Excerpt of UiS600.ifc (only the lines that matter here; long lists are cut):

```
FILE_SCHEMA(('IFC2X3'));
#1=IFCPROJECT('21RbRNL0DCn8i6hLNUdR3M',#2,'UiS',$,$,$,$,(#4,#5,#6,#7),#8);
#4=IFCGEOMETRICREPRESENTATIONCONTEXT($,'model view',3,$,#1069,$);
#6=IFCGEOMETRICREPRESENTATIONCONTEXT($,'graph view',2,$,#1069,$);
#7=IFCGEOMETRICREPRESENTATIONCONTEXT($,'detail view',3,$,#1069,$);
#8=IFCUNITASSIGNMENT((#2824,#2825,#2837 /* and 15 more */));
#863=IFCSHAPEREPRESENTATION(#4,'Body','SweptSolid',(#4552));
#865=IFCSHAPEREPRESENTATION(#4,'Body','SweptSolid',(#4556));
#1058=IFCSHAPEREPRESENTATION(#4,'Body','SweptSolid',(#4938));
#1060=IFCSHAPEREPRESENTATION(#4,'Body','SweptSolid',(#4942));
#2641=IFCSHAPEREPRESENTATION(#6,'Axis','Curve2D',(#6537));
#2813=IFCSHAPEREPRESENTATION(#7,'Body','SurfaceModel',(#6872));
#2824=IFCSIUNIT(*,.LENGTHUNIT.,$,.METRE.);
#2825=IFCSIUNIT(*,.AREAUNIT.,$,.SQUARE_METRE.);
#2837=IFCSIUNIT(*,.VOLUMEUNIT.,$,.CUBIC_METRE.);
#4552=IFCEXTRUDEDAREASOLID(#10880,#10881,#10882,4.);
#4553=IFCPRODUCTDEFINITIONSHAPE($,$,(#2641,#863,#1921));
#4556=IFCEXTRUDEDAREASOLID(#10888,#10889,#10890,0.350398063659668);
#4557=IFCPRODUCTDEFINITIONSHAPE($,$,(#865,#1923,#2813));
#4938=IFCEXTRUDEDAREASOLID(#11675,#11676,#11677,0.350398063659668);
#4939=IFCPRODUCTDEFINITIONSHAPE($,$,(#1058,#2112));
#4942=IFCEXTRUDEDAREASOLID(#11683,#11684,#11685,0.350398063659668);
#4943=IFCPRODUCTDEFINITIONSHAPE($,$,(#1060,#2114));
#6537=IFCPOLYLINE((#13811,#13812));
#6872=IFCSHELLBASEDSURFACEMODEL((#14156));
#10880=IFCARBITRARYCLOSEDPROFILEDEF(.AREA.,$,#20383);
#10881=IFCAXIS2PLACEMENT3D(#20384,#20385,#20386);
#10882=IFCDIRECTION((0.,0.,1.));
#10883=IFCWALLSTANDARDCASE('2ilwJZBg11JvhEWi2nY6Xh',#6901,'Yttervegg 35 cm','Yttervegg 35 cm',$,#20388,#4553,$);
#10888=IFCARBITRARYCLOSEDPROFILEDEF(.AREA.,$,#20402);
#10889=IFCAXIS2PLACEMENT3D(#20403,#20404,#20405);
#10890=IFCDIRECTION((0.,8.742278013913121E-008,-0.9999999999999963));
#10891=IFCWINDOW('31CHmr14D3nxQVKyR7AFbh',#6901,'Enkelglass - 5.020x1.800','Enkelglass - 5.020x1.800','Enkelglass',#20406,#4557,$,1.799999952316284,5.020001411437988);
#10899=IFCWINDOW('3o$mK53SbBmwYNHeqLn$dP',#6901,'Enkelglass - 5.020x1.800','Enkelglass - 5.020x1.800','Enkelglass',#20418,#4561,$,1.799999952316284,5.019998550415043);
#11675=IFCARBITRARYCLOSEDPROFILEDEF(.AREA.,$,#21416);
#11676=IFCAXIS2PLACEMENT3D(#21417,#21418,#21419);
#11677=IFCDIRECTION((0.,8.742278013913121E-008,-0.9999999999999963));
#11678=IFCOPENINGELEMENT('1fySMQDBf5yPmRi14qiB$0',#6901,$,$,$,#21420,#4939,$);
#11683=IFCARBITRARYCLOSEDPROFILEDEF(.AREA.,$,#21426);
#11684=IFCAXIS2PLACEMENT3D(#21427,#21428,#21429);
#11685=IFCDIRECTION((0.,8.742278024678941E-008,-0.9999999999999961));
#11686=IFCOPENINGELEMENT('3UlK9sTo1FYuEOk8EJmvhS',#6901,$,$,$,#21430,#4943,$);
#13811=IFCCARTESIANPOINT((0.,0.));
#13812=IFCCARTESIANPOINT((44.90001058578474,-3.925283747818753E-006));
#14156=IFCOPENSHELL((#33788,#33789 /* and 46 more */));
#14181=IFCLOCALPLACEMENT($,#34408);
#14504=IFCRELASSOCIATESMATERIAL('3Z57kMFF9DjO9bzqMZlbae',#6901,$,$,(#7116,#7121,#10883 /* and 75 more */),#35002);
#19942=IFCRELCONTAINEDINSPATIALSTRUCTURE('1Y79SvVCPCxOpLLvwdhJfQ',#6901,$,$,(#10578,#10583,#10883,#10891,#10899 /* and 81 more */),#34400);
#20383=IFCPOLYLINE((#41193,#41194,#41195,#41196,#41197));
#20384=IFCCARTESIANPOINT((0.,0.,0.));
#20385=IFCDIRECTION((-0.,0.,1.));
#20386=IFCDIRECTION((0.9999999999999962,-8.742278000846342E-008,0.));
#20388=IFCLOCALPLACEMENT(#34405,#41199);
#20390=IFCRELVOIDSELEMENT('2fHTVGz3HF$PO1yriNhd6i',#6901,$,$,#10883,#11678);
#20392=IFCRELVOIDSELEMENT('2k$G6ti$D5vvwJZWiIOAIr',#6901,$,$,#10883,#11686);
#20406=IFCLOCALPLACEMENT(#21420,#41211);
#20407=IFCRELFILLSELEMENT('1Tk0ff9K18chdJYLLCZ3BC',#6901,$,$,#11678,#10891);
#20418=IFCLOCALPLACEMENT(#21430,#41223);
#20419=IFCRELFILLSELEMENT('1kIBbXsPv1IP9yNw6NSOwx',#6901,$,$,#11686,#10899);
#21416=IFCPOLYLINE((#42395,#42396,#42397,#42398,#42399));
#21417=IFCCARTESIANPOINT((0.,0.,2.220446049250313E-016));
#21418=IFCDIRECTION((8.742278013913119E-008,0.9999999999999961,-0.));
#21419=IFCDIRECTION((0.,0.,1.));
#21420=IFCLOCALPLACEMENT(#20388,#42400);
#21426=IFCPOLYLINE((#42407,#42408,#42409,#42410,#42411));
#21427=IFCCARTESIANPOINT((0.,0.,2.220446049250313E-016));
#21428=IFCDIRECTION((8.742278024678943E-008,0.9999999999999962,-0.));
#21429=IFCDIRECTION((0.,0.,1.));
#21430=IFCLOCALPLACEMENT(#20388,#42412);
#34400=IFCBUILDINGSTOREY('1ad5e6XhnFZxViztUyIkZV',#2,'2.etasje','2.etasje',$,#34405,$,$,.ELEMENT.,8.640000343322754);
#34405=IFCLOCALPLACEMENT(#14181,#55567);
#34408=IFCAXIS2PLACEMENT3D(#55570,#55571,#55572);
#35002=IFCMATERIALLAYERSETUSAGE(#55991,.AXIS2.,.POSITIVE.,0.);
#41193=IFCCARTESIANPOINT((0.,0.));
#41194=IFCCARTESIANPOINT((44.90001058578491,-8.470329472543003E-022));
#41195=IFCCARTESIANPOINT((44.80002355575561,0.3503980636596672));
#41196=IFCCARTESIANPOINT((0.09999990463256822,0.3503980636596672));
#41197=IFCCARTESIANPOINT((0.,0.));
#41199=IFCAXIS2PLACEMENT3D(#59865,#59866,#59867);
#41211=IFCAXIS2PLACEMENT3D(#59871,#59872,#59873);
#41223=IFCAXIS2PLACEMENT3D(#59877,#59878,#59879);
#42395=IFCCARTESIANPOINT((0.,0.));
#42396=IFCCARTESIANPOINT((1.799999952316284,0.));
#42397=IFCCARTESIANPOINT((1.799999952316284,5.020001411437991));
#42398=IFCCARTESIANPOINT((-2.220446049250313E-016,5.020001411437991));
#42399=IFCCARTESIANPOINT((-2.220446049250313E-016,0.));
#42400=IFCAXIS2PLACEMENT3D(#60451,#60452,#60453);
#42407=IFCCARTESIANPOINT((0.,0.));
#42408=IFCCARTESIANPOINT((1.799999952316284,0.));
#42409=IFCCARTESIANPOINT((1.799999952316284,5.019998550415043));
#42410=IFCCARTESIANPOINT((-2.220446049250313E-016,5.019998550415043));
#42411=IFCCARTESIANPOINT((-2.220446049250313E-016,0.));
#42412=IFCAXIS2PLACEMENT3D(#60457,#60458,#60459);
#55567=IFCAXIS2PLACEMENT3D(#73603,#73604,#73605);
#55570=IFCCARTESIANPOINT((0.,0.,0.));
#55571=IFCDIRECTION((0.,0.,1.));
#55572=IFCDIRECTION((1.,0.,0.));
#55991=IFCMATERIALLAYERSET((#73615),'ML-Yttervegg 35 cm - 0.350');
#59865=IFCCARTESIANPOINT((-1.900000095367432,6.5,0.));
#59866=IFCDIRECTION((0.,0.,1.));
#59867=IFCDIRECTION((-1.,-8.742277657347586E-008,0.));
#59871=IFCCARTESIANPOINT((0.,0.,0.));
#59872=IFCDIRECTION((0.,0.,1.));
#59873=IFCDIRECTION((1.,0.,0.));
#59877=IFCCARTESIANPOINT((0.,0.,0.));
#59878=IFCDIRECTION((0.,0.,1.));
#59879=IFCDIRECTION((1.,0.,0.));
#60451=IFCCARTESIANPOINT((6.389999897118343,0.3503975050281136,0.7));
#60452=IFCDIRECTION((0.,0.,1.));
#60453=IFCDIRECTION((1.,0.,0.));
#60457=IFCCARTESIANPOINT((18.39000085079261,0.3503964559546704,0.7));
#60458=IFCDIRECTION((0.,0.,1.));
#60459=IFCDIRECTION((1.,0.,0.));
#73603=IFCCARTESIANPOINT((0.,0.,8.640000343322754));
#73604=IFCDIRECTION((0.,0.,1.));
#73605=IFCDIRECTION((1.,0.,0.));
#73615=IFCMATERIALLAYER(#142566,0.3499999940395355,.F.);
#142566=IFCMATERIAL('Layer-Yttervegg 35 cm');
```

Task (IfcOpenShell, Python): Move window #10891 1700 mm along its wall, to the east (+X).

```python
import ifcopenshell
import ifcopenshell.api.geometry
import ifcopenshell.util.placement

model = ifcopenshell.open("UiS600.ifc")

window = model.by_id(10891)
opening = window.FillsVoids[0].RelatingOpeningElement
wall = opening.VoidsElements[0].RelatingBuildingElement

wall_matrix = ifcopenshell.util.placement.get_local_placement(wall.ObjectPlacement)
shift = wall_matrix[:3, 0] * -1.7
before = ifcopenshell.util.placement.get_local_placement(window.ObjectPlacement)[:3, 3].copy()

# The window is placed relative to its opening, so it follows when the opening moves.
matrix = ifcopenshell.util.placement.get_local_placement(opening.ObjectPlacement)
matrix[:3, 3] += shift
ifcopenshell.api.geometry.edit_object_placement(
    model, product=opening, matrix=matrix, is_si=False, should_transform_children=True
)

after = ifcopenshell.util.placement.get_local_placement(window.ObjectPlacement)[:3, 3]
print("window moved by", (after - before).round(3) + 0.0)

model.write("UiS600_updated.ifc")
```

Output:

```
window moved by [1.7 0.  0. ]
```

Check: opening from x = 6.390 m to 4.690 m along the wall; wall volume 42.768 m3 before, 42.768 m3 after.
